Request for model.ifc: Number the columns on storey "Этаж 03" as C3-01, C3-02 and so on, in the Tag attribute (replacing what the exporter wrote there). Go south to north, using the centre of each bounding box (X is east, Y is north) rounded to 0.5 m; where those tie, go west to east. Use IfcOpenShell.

First a look at what the model holds.

```python
import ifcopenshell
import ifcopenshell.util.element
import ifcopenshell.util.placement

model = ifcopenshell.open("model.ifc")
print(model.schema)
storey = next(s for s in model.by_type("IfcBuildingStorey") if s.Name == "Этаж 03")
columns = [e for e in ifcopenshell.util.element.get_decomposition(storey) if e.is_a("IfcColumn")]
for e in sorted(columns, key=lambda e: e.id()):
    origin = ifcopenshell.util.placement.get_local_placement(e.ObjectPlacement)[:3, 3]
    print(e.id(), e.Tag, e.Name, origin.round(2) + 0.0, sep=" | ")
```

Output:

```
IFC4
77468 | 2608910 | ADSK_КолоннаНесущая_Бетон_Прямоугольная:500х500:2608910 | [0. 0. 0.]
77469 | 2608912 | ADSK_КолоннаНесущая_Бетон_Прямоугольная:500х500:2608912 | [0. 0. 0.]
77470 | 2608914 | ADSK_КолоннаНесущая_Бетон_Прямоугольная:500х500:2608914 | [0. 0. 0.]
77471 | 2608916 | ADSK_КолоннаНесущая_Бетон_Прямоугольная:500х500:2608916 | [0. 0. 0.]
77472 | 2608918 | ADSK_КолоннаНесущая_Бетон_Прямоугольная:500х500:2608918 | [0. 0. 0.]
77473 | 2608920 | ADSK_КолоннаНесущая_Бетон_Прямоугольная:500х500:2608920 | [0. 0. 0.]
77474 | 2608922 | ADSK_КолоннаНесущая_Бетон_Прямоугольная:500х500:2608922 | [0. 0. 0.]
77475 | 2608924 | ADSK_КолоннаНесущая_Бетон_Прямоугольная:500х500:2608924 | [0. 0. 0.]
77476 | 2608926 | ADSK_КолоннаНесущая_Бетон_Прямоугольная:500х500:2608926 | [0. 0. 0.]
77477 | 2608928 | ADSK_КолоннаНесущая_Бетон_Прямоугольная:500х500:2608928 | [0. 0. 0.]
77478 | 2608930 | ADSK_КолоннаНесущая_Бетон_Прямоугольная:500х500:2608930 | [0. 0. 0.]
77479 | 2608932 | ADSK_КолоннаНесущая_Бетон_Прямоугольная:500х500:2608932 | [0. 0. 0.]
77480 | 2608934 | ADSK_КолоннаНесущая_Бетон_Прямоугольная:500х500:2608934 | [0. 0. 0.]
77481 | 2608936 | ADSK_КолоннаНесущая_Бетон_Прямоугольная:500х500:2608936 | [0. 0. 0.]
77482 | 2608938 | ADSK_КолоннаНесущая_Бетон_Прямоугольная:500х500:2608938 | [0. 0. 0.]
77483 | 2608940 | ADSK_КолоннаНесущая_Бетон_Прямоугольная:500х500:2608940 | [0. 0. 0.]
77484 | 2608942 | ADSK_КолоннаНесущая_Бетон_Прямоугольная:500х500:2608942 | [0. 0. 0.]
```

```python
import ifcopenshell
import ifcopenshell.geom
import ifcopenshell.util.element
import ifcopenshell.util.shape

model = ifcopenshell.open("model.ifc")
settings = ifcopenshell.geom.settings()
settings.set("use-world-coords", True)


def centre(element):
    shape = ifcopenshell.geom.create_shape(settings, element)
    return ifcopenshell.util.shape.get_bbox_centroid(shape.geometry)


storey = next(s for s in model.by_type("IfcBuildingStorey") if s.Name == "Этаж 03")
columns = [e for e in ifcopenshell.util.element.get_decomposition(storey) if e.is_a("IfcColumn")]

# Insertion points can sit at a corner or the storey origin, so sort by the geometry (in metres).
centres = {e: centre(e) for e in columns}
columns.sort(key=lambda e: (round(centres[e][1] / 0.5), centres[e][0]))

for i, e in enumerate(columns, start=1):
    number = f"C3-{i:02d}"
    e.Tag = number
    print(e.id(), number)

model.write("model_updated.ifc")
```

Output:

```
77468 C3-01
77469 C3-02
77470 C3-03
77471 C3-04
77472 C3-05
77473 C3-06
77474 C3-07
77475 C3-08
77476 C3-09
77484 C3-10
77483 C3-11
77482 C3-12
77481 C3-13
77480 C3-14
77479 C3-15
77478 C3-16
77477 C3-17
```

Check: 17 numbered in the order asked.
